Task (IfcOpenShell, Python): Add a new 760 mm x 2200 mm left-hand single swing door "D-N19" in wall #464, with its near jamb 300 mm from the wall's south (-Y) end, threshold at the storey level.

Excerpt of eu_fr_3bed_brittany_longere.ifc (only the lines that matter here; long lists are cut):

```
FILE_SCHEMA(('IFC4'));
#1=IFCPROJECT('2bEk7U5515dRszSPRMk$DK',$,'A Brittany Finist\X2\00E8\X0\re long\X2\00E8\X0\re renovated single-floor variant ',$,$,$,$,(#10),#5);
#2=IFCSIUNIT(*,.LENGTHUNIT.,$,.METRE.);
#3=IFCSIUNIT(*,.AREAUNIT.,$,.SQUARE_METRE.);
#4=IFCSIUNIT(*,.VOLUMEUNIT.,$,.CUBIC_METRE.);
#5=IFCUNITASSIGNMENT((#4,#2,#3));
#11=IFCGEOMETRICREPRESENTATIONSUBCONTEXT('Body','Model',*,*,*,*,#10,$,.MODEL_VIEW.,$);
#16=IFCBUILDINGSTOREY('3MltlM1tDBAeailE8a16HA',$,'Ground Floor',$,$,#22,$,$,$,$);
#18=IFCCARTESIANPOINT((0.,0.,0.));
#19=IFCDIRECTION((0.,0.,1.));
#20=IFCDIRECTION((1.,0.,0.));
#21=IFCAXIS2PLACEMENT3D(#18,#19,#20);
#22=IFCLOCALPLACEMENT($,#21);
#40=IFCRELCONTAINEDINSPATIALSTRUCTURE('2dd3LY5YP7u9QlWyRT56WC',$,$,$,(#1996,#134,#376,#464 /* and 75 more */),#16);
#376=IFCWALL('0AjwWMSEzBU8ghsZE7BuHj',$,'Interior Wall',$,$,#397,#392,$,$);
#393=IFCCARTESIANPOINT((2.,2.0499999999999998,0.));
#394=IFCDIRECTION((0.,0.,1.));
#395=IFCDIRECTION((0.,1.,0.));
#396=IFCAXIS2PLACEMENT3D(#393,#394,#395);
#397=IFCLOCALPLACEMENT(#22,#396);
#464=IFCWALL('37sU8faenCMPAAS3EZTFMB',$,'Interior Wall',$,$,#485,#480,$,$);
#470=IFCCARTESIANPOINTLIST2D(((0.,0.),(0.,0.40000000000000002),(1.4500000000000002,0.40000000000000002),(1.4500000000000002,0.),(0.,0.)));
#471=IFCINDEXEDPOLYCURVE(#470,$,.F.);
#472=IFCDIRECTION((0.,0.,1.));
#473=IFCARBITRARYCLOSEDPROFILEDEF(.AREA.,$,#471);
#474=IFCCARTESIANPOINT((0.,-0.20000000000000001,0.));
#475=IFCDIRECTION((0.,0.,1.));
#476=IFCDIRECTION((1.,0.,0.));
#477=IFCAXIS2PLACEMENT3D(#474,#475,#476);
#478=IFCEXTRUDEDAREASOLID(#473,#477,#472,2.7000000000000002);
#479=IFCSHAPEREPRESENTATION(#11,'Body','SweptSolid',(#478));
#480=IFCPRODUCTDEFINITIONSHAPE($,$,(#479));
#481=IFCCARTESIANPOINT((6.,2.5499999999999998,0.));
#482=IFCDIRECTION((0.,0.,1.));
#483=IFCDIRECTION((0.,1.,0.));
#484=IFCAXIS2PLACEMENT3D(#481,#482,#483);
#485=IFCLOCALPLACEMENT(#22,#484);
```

```python
import numpy as np
import ifcopenshell
import ifcopenshell.api.feature
import ifcopenshell.api.geometry
import ifcopenshell.api.root
import ifcopenshell.api.spatial
import ifcopenshell.geom
import ifcopenshell.util.element
import ifcopenshell.util.placement
import ifcopenshell.util.representation
import ifcopenshell.util.shape
import ifcopenshell.util.unit

model = ifcopenshell.open("eu_fr_3bed_brittany_longere.ifc")
unit_scale = ifcopenshell.util.unit.calculate_unit_scale(model)
settings = ifcopenshell.geom.settings()


def volume(element):
    """Net volume in cubic metres, openings subtracted."""
    shape = ifcopenshell.geom.create_shape(settings, element)
    return ifcopenshell.util.shape.get_volume(shape.geometry)


wall = model.by_guid("37sU8faenCMPAAS3EZTFMB")
storey = ifcopenshell.util.element.get_container(wall, ifc_class="IfcBuildingStorey")
context = ifcopenshell.util.representation.get_context(model, "Model", "Body", "MODEL_VIEW")
before = volume(wall)

width, height, from_end, sill = 0.76, 2.2, 0.3, 0.0  # metres

# The wall runs along its own X axis, and the end named is its -X end.
wall_shape = ifcopenshell.geom.create_shape(settings, wall)
x, y, z = ifcopenshell.util.shape.get_vertices(wall_shape.geometry).T
start = x.min() + from_end
face, thickness = float(y.min()), float(y.max() - y.min())
wall_matrix = ifcopenshell.util.placement.get_local_placement(wall.ObjectPlacement)
level = ifcopenshell.util.placement.get_local_placement(storey.ObjectPlacement)[2, 3]


def in_wall(x, y):
    """Placement at x, y metres in the wall's axes, at sill height."""
    matrix = wall_matrix.copy()
    matrix[:, 3] = wall_matrix @ np.array([x / unit_scale, y / unit_scale, 0.0, 1.0])
    matrix[2, 3] = level + sill / unit_scale
    return matrix


# Opening: a box that overshoots both wall faces by 50 mm.
opening = ifcopenshell.api.root.create_entity(model, ifc_class="IfcOpeningElement", predefined_type="OPENING")
box = ifcopenshell.api.geometry.add_wall_representation(
    model, context=context, length=width, height=height, thickness=thickness + 0.1
)
ifcopenshell.api.geometry.assign_representation(model, product=opening, representation=box)
ifcopenshell.api.geometry.edit_object_placement(model, product=opening, matrix=in_wall(start, face - 0.05), is_si=False)
ifcopenshell.api.feature.add_feature(model, feature=opening, element=wall)

door = ifcopenshell.api.root.create_entity(model, ifc_class="IfcDoor", name="D-N19", predefined_type="DOOR")
door.OverallWidth, door.OverallHeight = width / unit_scale, height / unit_scale
door.OperationType = "SINGLE_SWING_LEFT"
body = ifcopenshell.api.geometry.add_door_representation(
    model,
    context=context,
    overall_width=door.OverallWidth,
    overall_height=door.OverallHeight,
    operation_type="SINGLE_SWING_LEFT",
    lining_properties={"LiningDepth": thickness / unit_scale, "ThresholdDepth": thickness / unit_scale},
)
ifcopenshell.api.geometry.assign_representation(model, product=door, representation=body)
ifcopenshell.api.spatial.assign_container(model, products=[door], relating_structure=storey)
ifcopenshell.api.feature.add_filling(model, opening=opening, element=door)

# The lining spans the wall, so the door starts at the wall face.
ifcopenshell.api.geometry.edit_object_placement(model, product=door, matrix=in_wall(start, face), is_si=False)

after = volume(wall)

print(f"wall volume {before:.3f} -> {after:.3f} m3")

model.write("eu_fr_3bed_brittany_longere_updated.ifc")
```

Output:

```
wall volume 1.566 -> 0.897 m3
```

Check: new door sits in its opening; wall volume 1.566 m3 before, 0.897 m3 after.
